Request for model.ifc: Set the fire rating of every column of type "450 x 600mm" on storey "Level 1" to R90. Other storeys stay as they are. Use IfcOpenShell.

First a look at what the model holds.

```python
import ifcopenshell
import ifcopenshell.util.element

model = ifcopenshell.open("model.ifc")
print(model.schema)
storey = next(s for s in model.by_type("IfcBuildingStorey") if s.Name == "Level 1")
columns = [e for e in ifcopenshell.util.element.get_decomposition(storey) if e.is_a("IfcColumn")]
seen = {}
for e in columns:
    element_type = ifcopenshell.util.element.get_type(e)
    key = (element_type.Name if element_type != e and element_type else None, ifcopenshell.util.element.get_pset(e, "Pset_ColumnCommon", "FireRating"))
    seen[key] = seen.get(key, 0) + 1
for (name, value), count in sorted(seen.items(), key=str):
    print(count, "x", name, "|", value)
```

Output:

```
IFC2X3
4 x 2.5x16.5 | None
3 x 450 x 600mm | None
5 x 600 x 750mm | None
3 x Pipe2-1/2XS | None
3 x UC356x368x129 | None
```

```python
import ifcopenshell
import ifcopenshell.api.pset
import ifcopenshell.util.element

model = ifcopenshell.open("model.ifc")

storey = next(s for s in model.by_type("IfcBuildingStorey") if s.Name == "Level 1")
columns = [e for e in ifcopenshell.util.element.get_decomposition(storey) if e.is_a("IfcColumn")]

count = 0
for e in columns:
    element_type = ifcopenshell.util.element.get_type(e)
    if element_type in (None, e) or element_type.Name != "450 x 600mm":
        continue
    # add_pset returns the element's existing set when there is one.
    pset = ifcopenshell.api.pset.add_pset(model, product=e, name="Pset_ColumnCommon")
    ifcopenshell.api.pset.edit_pset(model, pset=pset, properties={"FireRating": "R90"})
    count += 1

print(count, "columns updated")

model.write("model-out.ifc")
```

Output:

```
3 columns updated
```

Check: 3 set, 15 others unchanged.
